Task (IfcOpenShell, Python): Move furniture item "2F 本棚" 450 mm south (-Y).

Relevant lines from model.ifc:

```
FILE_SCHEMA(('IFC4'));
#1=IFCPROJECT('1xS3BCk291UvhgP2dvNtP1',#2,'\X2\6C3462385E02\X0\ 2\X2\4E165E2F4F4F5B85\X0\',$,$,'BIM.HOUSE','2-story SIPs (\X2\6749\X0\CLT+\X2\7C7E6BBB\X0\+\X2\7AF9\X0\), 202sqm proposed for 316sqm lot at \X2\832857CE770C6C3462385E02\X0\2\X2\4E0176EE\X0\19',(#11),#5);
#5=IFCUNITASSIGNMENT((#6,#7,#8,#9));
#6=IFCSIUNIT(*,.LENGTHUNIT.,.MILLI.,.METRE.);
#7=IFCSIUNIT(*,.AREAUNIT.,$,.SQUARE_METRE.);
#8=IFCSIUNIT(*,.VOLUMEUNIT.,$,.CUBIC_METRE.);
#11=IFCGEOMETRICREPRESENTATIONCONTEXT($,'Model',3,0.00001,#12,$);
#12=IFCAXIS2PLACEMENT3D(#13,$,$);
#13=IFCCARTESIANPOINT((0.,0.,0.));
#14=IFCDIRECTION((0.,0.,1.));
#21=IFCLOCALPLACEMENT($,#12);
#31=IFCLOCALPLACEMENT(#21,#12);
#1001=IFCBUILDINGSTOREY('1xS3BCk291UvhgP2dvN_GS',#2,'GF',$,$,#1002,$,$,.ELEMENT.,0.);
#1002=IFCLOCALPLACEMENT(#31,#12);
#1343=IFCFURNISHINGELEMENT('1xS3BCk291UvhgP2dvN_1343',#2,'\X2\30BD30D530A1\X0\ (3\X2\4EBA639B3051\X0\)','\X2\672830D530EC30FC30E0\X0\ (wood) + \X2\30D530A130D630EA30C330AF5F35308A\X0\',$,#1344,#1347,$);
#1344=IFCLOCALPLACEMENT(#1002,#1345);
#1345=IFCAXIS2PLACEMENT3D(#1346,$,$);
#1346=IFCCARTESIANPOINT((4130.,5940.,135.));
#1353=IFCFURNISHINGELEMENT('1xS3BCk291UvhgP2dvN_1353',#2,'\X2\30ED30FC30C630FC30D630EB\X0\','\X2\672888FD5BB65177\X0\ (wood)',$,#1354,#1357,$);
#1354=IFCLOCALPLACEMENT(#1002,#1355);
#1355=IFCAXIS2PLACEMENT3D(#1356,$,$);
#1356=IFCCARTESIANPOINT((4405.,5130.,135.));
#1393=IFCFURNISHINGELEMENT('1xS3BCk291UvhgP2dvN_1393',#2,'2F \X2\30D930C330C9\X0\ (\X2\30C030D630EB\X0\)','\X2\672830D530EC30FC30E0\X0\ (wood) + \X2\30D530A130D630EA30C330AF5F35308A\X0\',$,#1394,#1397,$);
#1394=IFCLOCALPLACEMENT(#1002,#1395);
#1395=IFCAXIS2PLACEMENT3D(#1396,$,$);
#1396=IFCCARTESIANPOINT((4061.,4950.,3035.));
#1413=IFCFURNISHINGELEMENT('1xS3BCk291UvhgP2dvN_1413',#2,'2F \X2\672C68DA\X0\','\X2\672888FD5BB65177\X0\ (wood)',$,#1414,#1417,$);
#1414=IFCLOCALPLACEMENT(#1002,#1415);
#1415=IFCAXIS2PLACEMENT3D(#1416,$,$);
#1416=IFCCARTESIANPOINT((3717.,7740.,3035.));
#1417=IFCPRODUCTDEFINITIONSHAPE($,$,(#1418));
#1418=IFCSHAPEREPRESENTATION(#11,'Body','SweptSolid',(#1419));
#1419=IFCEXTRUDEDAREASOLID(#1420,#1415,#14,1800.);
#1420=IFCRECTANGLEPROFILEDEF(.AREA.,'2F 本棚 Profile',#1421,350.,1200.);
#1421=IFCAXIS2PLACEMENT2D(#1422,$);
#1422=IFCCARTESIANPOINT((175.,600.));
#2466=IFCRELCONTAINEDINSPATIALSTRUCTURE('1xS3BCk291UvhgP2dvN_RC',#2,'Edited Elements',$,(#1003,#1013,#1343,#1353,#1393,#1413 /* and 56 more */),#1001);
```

```python
import ifcopenshell
import ifcopenshell.api.geometry
import ifcopenshell.util.placement
import ifcopenshell.util.unit

model = ifcopenshell.open("model.ifc")
unit_scale = ifcopenshell.util.unit.calculate_unit_scale(model)

item = model.by_guid("1xS3BCk291UvhgP2dvN_1413")
matrix = ifcopenshell.util.placement.get_local_placement(item.ObjectPlacement)
matrix[1, 3] -= 0.45 / unit_scale
ifcopenshell.api.geometry.edit_object_placement(model, product=item, matrix=matrix, is_si=False)

print(ifcopenshell.util.placement.get_local_placement(item.ObjectPlacement).round(3) + 0.0)

model.write("model-out.ifc")
```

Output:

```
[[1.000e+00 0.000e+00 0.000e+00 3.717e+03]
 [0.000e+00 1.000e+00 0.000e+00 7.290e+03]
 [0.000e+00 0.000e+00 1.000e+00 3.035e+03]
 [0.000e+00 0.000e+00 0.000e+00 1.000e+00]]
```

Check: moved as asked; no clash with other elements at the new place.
